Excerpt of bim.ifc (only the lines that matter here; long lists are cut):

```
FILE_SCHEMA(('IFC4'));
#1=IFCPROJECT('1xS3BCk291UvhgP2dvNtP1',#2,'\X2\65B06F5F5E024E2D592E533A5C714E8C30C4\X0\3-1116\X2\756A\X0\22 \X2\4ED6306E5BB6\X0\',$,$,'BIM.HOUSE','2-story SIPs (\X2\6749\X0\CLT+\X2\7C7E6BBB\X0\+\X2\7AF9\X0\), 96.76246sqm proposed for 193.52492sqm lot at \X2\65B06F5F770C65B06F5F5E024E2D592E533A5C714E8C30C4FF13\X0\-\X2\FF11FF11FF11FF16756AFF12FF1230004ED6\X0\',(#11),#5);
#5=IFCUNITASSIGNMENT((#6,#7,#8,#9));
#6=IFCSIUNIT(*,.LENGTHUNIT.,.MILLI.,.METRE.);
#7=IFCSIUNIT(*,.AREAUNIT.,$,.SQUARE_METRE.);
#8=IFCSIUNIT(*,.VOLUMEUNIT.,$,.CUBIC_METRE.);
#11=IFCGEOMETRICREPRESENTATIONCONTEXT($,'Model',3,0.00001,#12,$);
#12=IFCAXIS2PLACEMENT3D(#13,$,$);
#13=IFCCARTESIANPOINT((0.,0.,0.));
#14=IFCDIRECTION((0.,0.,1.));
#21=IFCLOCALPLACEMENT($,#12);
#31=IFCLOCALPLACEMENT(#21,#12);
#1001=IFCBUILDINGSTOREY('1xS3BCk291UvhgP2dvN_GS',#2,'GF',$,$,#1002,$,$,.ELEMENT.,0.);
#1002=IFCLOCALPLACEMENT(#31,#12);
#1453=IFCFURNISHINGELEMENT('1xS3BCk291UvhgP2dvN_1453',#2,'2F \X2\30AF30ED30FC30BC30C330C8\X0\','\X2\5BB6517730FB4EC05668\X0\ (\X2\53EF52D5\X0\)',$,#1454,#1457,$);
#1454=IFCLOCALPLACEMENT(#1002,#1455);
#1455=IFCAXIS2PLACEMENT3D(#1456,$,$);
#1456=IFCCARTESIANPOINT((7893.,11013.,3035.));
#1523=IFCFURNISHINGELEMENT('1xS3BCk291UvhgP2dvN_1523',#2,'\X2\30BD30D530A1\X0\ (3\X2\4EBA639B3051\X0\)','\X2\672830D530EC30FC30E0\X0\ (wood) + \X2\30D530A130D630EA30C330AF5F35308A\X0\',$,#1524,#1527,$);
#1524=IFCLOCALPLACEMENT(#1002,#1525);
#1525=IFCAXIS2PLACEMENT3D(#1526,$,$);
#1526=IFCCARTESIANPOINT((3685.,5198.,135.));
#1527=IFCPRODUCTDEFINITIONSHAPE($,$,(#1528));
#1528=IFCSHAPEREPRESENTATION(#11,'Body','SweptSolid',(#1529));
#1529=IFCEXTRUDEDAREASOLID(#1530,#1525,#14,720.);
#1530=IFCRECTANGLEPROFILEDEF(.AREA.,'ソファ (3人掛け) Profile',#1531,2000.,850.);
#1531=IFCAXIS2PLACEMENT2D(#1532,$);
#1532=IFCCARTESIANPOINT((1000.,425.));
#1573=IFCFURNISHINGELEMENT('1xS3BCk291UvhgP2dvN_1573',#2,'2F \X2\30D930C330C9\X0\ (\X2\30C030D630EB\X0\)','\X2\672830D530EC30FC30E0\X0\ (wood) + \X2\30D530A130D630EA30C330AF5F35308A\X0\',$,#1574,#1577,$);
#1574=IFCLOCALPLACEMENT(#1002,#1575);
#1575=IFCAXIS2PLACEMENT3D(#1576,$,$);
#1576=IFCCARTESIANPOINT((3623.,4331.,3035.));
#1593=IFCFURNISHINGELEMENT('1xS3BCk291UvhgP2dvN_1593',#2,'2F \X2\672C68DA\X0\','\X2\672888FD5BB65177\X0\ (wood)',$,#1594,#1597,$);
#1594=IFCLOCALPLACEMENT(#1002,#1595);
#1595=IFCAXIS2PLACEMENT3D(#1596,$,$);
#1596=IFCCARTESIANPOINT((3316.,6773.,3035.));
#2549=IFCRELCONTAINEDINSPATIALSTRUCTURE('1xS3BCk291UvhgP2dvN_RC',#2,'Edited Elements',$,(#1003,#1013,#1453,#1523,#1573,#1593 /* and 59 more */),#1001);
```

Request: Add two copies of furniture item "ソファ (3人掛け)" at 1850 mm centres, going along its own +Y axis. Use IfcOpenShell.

```python
import ifcopenshell
import ifcopenshell.api.geometry
import ifcopenshell.api.root
import ifcopenshell.util.element
import ifcopenshell.util.placement
import ifcopenshell.util.unit

model = ifcopenshell.open("bim.ifc")
unit_scale = ifcopenshell.util.unit.calculate_unit_scale(model)


def reuse_history(source, copy):
    """copy_class also copies each property set's owner history, people and application; keep the originals."""
    for rel in copy.IsDefinedBy:
        if rel.is_a("IfcRelDefinesByProperties") and (history := rel.RelatingPropertyDefinition.OwnerHistory):
            rel.RelatingPropertyDefinition.OwnerHistory = source.OwnerHistory
            ifcopenshell.util.element.remove_deep2(model, history)


source = model.by_guid("1xS3BCk291UvhgP2dvN_1523")
base = ifcopenshell.util.placement.get_local_placement(source.ObjectPlacement)
step = base[:3, 1] * 1.85 / unit_scale

for i in range(1, 3):
    copy = ifcopenshell.api.root.copy_class(model, product=source)
    copy.Representation = ifcopenshell.util.element.copy_deep(
        model, source.Representation, exclude=["IfcGeometricRepresentationContext", "IfcRepresentationMap"]
    )
    reuse_history(source, copy)
    matrix = base.copy()
    matrix[:3, 3] += i * step
    print("added at", matrix[:3, 3].round(3) + 0.0)
    ifcopenshell.api.geometry.edit_object_placement(model, product=copy, matrix=matrix, is_si=False)

model.write("bim_rev.ifc")
```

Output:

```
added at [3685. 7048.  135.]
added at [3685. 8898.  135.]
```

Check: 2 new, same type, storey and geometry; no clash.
